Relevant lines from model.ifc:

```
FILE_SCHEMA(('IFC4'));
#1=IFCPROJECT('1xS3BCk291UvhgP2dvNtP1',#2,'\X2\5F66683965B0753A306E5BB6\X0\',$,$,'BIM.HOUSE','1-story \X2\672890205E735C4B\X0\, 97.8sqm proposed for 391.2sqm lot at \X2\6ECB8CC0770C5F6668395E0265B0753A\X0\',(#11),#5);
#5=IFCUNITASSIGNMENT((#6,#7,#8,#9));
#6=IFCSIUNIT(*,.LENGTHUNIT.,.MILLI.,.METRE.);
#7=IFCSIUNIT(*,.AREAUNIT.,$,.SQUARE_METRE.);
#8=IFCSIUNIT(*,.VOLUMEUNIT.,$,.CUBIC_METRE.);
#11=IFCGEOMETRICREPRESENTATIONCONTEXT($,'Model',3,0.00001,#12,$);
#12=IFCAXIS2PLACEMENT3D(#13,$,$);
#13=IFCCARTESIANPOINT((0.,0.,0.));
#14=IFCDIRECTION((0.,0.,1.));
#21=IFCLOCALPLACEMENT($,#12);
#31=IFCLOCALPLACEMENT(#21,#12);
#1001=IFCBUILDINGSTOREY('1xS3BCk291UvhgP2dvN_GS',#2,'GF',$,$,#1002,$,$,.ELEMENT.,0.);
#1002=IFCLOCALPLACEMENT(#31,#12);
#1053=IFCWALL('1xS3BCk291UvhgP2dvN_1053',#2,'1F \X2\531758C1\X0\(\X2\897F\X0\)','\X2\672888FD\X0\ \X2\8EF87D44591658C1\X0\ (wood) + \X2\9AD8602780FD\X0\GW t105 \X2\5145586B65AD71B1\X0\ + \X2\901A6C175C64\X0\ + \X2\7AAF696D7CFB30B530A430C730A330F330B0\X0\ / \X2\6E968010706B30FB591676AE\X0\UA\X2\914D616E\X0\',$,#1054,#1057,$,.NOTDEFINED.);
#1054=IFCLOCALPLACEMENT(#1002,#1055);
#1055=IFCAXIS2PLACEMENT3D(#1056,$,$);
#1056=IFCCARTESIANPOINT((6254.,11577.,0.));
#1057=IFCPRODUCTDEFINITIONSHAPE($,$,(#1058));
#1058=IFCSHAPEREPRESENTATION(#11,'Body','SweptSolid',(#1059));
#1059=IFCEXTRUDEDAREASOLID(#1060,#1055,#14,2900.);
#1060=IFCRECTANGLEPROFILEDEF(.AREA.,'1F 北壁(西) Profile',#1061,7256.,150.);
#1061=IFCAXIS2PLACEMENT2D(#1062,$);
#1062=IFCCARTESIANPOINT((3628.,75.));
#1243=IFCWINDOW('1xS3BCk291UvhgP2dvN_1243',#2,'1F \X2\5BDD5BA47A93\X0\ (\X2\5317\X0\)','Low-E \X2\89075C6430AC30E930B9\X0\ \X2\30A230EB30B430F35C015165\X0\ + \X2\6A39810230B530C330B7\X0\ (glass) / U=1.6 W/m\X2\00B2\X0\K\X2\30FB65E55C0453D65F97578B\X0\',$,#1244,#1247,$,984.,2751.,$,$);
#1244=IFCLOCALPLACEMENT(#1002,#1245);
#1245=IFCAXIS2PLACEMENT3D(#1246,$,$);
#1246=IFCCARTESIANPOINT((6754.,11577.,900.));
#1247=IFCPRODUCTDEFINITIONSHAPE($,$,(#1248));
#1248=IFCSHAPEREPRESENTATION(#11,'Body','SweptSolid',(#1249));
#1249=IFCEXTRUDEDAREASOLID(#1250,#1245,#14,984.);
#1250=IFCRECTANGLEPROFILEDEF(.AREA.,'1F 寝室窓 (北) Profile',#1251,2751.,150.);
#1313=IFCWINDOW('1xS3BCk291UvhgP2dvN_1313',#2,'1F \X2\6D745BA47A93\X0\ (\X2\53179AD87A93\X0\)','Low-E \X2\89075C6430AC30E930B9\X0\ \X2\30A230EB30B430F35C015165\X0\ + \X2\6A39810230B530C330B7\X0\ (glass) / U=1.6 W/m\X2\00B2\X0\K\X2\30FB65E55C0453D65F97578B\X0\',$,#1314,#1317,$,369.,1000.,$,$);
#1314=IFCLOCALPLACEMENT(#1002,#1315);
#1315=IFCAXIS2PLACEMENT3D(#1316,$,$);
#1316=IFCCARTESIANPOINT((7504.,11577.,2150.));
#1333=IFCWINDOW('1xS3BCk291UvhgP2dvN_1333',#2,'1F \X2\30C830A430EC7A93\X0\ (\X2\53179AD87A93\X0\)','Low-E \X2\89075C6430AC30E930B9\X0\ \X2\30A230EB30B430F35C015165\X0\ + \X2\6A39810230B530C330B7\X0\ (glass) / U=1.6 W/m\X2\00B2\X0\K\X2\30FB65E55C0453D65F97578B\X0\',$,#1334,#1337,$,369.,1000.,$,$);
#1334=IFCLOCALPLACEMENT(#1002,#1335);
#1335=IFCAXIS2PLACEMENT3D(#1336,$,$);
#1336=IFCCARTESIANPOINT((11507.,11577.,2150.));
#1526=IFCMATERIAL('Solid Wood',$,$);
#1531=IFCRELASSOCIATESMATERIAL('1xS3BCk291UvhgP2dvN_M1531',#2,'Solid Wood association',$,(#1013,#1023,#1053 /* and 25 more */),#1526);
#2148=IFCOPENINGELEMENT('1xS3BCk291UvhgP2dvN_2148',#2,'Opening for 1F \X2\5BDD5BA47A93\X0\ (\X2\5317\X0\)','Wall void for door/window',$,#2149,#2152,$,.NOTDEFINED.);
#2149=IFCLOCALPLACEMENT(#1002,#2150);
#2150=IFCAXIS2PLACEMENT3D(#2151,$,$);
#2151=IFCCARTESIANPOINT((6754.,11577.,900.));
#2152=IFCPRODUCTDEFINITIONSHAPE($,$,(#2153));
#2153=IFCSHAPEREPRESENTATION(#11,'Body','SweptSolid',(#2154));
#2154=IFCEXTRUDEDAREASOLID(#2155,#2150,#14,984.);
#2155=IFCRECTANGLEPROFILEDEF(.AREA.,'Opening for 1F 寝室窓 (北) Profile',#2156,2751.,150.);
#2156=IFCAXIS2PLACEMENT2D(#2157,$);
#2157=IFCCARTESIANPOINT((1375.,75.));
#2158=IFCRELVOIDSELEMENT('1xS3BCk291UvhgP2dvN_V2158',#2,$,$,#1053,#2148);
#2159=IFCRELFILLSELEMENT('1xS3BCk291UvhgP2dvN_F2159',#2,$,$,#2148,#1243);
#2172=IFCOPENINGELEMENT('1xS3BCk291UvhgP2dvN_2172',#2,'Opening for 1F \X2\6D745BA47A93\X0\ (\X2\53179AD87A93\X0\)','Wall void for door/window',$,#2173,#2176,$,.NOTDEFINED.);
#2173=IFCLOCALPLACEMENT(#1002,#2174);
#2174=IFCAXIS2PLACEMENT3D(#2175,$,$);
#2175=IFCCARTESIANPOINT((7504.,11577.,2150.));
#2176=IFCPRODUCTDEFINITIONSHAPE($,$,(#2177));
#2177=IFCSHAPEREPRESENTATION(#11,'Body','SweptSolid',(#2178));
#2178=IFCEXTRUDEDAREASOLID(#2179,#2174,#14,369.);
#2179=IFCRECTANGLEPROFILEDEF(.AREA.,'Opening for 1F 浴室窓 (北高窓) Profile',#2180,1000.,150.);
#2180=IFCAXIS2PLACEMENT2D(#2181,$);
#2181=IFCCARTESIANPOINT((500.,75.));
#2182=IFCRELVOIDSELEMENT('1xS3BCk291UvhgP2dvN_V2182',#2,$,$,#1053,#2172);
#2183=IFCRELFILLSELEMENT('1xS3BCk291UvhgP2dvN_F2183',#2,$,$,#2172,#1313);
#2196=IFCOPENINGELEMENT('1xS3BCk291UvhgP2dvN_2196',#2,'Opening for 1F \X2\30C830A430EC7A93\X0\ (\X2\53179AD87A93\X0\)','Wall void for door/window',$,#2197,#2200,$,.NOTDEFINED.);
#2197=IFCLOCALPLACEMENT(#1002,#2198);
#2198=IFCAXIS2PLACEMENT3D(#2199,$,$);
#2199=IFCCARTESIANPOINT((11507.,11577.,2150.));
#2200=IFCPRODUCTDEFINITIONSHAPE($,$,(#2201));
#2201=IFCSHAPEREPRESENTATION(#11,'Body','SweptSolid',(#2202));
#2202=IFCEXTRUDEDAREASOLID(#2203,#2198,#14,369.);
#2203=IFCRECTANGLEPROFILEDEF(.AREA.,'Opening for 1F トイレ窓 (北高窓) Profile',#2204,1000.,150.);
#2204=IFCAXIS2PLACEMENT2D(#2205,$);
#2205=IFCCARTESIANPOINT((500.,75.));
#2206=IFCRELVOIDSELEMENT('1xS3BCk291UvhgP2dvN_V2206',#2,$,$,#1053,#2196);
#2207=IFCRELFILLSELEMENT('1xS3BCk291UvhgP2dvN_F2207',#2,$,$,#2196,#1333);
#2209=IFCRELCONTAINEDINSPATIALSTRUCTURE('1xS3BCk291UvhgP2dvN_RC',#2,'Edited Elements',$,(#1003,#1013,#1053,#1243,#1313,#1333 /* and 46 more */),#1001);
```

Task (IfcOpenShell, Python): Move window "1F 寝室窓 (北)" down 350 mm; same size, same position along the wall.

```python
import numpy as np
import ifcopenshell
import ifcopenshell.api.geometry
import ifcopenshell.util.placement
import ifcopenshell.util.unit

model = ifcopenshell.open("model.ifc")
unit_scale = ifcopenshell.util.unit.calculate_unit_scale(model)

window = model.by_guid("1xS3BCk291UvhgP2dvN_1243")
opening = window.FillsVoids[0].RelatingOpeningElement
dz = -350.0

shift = np.array([0.0, 0.0, dz])
# The window is not placed relative to its opening, so move both.
for product in (opening, window):
    matrix = ifcopenshell.util.placement.get_local_placement(product.ObjectPlacement)
    matrix[:3, 3] += shift
    ifcopenshell.api.geometry.edit_object_placement(model, product=product, matrix=matrix, is_si=False)

print(f"moved by {dz * unit_scale:+.3f} m")

model.write("model_edited.ifc")
```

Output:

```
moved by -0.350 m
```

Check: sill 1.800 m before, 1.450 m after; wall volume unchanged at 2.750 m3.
